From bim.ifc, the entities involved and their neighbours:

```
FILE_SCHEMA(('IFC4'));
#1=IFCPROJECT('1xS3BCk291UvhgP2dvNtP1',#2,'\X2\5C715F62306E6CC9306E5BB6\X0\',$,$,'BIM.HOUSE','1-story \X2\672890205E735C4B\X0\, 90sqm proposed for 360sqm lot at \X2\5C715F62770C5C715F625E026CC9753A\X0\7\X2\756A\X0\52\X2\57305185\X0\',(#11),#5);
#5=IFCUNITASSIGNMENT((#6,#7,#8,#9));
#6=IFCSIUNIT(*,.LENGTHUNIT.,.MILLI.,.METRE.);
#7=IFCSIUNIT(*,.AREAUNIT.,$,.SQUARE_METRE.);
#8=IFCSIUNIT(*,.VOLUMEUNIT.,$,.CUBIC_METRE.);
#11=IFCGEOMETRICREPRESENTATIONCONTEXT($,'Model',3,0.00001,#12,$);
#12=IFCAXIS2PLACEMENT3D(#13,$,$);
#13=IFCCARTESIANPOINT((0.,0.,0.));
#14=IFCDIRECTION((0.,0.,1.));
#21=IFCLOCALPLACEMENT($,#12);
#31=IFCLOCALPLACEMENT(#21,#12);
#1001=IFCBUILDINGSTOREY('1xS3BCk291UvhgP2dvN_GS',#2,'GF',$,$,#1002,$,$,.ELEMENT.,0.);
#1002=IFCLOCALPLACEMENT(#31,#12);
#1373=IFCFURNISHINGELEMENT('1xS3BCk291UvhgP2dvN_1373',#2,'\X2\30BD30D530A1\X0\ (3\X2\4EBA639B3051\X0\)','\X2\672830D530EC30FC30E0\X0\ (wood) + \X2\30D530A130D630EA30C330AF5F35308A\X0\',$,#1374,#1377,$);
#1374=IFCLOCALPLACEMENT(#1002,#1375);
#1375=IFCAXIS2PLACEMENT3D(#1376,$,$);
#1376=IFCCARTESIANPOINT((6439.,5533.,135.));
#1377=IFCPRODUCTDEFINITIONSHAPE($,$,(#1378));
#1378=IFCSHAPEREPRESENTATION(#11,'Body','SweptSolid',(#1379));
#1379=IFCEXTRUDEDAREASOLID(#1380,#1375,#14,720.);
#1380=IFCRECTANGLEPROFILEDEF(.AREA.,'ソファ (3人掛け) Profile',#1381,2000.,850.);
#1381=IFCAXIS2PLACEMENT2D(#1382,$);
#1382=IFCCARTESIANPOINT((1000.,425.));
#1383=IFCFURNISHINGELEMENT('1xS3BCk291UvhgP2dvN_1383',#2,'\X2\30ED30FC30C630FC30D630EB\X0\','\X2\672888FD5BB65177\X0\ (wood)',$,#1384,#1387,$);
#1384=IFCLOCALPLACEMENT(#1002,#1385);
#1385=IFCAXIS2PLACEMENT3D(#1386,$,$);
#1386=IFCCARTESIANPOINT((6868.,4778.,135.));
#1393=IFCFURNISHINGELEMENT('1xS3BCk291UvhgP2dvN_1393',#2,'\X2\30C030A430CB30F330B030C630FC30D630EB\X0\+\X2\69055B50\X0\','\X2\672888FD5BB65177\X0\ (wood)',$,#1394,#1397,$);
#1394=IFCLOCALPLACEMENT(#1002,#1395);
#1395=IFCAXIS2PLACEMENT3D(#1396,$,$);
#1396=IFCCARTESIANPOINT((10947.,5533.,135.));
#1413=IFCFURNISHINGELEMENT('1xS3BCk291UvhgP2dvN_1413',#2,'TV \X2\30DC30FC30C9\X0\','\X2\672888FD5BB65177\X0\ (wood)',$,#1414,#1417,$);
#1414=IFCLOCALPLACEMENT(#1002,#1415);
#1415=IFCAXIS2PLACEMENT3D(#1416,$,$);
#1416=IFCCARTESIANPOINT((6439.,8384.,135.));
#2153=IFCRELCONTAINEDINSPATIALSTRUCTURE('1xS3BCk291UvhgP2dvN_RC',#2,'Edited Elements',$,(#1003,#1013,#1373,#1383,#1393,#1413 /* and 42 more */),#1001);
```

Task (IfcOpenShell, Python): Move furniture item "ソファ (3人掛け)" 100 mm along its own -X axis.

```python
import ifcopenshell
import ifcopenshell.api.geometry
import ifcopenshell.util.placement
import ifcopenshell.util.unit

model = ifcopenshell.open("bim.ifc")
unit_scale = ifcopenshell.util.unit.calculate_unit_scale(model)

item = model.by_guid("1xS3BCk291UvhgP2dvN_1373")
matrix = ifcopenshell.util.placement.get_local_placement(item.ObjectPlacement)
matrix[:3, 3] -= matrix[:3, 0] * 0.1 / unit_scale
ifcopenshell.api.geometry.edit_object_placement(model, product=item, matrix=matrix, is_si=False)

print(ifcopenshell.util.placement.get_local_placement(item.ObjectPlacement).round(3) + 0.0)

model.write("bim_edited.ifc")
```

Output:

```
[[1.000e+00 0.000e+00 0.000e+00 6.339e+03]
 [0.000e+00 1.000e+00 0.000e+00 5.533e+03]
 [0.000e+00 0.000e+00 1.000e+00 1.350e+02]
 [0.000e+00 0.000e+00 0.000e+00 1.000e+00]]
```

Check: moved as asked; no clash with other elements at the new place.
